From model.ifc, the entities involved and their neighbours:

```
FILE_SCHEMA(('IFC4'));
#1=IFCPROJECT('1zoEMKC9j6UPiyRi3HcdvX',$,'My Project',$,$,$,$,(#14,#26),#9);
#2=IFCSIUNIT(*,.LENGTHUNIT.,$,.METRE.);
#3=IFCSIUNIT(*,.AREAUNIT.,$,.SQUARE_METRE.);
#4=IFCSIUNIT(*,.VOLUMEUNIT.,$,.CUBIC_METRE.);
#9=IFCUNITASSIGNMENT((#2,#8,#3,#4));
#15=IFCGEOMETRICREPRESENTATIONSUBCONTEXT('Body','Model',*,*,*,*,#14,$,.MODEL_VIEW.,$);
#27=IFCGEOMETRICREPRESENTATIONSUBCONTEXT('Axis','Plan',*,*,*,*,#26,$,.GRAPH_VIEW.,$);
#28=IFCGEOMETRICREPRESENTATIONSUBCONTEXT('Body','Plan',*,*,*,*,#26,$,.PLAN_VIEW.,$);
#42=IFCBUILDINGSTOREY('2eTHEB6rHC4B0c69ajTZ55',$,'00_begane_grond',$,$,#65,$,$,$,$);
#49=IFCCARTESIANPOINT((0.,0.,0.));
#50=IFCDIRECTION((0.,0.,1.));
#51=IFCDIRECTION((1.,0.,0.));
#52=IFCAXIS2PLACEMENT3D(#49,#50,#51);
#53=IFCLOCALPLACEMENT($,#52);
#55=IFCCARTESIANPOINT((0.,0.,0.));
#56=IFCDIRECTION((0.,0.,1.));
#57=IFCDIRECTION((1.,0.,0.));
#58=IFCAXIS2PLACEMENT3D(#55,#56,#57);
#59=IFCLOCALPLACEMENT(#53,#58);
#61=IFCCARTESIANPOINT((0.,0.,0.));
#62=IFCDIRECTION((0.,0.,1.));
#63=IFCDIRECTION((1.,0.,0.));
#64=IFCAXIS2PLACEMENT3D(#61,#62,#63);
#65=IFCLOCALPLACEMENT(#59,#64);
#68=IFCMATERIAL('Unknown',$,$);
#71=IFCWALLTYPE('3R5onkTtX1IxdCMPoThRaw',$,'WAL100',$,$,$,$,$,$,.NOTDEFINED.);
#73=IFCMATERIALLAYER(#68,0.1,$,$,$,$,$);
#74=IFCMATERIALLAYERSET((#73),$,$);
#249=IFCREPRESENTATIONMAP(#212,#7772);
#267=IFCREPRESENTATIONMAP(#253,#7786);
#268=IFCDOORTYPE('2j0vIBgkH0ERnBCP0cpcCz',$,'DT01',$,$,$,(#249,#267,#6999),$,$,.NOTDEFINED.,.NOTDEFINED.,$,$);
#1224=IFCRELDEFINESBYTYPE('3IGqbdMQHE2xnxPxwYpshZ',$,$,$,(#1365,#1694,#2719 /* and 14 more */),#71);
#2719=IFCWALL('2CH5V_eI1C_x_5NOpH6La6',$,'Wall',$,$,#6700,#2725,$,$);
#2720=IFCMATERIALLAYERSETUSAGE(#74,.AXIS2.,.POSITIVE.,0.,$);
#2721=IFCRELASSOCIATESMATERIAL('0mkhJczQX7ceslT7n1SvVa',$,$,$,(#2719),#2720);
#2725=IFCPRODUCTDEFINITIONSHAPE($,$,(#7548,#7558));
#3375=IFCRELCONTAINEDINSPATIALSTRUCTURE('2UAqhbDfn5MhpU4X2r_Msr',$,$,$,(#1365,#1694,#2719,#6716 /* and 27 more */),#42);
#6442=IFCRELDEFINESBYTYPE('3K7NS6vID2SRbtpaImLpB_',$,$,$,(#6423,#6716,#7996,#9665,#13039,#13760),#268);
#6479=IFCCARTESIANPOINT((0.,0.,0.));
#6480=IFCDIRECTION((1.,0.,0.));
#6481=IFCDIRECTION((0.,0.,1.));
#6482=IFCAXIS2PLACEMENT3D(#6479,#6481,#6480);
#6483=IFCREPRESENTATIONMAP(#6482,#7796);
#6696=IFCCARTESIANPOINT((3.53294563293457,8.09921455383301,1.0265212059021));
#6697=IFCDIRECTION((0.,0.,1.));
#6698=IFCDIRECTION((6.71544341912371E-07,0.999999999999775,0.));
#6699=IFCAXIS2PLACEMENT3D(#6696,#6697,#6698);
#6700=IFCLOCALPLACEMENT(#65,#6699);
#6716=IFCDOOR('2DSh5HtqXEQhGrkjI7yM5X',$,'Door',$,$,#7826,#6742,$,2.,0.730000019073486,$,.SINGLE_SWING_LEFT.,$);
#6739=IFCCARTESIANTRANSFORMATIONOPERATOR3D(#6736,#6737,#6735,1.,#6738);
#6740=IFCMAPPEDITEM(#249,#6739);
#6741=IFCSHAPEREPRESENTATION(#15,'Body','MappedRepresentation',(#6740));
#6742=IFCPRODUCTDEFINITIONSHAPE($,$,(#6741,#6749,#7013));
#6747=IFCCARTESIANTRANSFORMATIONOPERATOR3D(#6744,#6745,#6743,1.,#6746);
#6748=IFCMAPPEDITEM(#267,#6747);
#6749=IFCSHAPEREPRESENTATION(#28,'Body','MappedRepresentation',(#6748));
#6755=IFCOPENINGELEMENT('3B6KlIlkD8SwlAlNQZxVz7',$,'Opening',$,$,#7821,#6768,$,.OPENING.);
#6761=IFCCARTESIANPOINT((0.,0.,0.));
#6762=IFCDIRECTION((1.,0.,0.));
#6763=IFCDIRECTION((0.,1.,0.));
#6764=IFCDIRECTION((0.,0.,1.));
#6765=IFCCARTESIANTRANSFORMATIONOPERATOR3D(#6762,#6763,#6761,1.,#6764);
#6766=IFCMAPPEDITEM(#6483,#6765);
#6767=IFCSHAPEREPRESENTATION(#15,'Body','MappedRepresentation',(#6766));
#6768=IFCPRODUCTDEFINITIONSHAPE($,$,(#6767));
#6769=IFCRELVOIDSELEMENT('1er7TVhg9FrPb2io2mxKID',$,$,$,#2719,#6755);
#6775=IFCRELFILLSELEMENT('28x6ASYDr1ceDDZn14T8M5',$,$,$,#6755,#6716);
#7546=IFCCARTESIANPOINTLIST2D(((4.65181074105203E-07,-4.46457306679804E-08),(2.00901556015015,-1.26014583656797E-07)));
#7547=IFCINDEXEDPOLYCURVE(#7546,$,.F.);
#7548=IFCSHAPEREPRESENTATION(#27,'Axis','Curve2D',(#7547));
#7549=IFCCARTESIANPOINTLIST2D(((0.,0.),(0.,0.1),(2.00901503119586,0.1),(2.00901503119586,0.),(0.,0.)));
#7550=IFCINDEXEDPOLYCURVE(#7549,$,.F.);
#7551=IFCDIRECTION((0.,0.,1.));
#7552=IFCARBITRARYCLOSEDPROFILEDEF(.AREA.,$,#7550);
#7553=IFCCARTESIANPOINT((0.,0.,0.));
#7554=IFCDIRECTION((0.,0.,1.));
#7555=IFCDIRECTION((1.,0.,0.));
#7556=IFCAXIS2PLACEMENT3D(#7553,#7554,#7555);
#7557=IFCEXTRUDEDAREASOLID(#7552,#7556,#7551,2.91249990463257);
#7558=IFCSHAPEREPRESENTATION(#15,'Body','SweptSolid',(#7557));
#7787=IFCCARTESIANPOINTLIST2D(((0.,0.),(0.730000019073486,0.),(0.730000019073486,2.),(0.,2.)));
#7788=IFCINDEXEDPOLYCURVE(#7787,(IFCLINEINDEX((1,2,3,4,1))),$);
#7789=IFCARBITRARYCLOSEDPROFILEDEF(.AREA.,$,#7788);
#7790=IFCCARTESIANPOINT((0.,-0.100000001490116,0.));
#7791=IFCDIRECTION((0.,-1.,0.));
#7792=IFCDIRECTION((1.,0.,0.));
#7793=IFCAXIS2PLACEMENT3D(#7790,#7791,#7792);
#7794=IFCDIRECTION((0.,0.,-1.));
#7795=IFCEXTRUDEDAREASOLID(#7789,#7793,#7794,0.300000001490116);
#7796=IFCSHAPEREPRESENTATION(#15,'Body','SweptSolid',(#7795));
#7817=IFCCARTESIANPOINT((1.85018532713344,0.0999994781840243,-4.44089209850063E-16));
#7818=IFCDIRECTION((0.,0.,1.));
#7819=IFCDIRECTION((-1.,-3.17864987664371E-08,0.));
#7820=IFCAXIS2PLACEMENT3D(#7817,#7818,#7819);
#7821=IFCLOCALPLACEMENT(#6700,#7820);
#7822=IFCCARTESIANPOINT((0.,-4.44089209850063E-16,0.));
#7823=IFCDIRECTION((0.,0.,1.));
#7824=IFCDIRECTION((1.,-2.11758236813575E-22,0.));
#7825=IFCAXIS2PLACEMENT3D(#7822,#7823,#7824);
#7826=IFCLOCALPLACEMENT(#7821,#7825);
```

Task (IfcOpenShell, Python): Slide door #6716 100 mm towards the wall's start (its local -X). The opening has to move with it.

```python
import ifcopenshell
import ifcopenshell.api.geometry
import ifcopenshell.util.placement
import ifcopenshell.util.unit

model = ifcopenshell.open("model.ifc")
unit_scale = ifcopenshell.util.unit.calculate_unit_scale(model)

door = model.by_guid("2DSh5HtqXEQhGrkjI7yM5X")
opening = door.FillsVoids[0].RelatingOpeningElement
wall = opening.VoidsElements[0].RelatingBuildingElement

wall_matrix = ifcopenshell.util.placement.get_local_placement(wall.ObjectPlacement)
shift = wall_matrix[:3, 0] * -0.1 / unit_scale
before = ifcopenshell.util.placement.get_local_placement(door.ObjectPlacement)[:3, 3].copy()

# The door is placed relative to its opening, so it follows when the opening moves.
matrix = ifcopenshell.util.placement.get_local_placement(opening.ObjectPlacement)
matrix[:3, 3] += shift
ifcopenshell.api.geometry.edit_object_placement(
    model, product=opening, matrix=matrix, is_si=False, should_transform_children=True
)

after = ifcopenshell.util.placement.get_local_placement(door.ObjectPlacement)[:3, 3]
print("door moved by", (after - before).round(3) + 0.0)

model.write("model_v2.ifc")
```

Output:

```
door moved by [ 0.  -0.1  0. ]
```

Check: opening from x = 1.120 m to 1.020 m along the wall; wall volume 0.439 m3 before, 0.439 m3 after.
